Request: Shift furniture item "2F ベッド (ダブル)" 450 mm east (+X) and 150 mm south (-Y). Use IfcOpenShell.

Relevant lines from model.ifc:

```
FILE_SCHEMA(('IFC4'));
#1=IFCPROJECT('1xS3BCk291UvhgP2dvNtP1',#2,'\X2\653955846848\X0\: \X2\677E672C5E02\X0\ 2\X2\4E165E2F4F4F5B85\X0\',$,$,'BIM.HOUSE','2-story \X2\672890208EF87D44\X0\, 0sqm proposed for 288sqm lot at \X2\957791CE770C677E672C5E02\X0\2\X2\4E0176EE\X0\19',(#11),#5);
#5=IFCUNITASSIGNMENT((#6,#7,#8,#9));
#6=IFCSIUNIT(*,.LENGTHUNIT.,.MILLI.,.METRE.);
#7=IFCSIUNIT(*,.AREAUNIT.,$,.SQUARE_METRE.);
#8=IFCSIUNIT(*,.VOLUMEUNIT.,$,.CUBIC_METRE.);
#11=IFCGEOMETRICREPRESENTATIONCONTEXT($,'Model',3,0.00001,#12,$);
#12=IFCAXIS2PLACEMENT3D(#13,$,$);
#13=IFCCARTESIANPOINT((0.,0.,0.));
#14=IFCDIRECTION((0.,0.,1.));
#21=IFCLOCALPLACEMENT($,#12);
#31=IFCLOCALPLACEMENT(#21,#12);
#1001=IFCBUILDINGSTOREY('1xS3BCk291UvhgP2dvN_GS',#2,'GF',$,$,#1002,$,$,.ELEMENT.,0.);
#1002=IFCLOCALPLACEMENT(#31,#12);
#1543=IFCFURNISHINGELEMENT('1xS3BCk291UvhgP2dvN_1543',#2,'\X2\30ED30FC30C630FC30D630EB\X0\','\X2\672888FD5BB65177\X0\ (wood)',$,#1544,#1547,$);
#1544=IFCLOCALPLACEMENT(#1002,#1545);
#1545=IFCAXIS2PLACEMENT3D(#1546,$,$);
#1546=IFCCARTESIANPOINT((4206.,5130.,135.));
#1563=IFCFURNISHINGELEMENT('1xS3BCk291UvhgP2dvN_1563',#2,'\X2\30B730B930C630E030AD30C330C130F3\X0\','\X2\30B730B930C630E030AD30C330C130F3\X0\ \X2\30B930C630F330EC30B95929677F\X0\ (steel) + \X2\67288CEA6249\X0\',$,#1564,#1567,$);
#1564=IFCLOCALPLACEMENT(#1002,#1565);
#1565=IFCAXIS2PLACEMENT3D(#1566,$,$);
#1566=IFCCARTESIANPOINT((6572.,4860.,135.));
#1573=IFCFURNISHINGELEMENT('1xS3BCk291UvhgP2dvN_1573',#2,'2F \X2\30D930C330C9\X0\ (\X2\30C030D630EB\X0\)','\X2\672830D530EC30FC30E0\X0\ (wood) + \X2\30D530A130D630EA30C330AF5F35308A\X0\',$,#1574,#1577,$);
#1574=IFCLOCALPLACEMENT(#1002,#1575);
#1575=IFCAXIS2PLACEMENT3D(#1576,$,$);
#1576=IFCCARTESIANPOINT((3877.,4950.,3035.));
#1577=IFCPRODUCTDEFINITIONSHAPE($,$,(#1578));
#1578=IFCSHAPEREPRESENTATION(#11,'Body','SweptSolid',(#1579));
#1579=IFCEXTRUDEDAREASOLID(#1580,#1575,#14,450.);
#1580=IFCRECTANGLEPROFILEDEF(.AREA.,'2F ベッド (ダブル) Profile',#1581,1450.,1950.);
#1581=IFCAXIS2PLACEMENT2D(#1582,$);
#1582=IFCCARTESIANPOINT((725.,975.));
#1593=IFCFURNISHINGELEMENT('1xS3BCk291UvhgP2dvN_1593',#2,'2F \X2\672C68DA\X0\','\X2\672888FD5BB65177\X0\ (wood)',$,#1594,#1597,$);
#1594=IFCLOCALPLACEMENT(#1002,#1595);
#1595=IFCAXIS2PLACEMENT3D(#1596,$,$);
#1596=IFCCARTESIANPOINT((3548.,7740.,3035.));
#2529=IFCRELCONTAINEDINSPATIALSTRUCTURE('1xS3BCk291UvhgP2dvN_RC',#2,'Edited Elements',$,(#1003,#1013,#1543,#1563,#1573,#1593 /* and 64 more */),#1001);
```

```python
import ifcopenshell
import ifcopenshell.api.geometry
import ifcopenshell.util.placement
import ifcopenshell.util.unit

model = ifcopenshell.open("model.ifc")
unit_scale = ifcopenshell.util.unit.calculate_unit_scale(model)

item = model.by_id(1573)
matrix = ifcopenshell.util.placement.get_local_placement(item.ObjectPlacement)
matrix[0, 3] += 0.45 / unit_scale
matrix[1, 3] -= 0.15 / unit_scale
ifcopenshell.api.geometry.edit_object_placement(model, product=item, matrix=matrix, is_si=False)

print(ifcopenshell.util.placement.get_local_placement(item.ObjectPlacement).round(3) + 0.0)

model.write("model_edited.ifc")
```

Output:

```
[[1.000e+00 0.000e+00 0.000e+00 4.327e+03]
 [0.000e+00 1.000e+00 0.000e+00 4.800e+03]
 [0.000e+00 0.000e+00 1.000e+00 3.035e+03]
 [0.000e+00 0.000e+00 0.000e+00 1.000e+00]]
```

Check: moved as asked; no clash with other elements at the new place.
